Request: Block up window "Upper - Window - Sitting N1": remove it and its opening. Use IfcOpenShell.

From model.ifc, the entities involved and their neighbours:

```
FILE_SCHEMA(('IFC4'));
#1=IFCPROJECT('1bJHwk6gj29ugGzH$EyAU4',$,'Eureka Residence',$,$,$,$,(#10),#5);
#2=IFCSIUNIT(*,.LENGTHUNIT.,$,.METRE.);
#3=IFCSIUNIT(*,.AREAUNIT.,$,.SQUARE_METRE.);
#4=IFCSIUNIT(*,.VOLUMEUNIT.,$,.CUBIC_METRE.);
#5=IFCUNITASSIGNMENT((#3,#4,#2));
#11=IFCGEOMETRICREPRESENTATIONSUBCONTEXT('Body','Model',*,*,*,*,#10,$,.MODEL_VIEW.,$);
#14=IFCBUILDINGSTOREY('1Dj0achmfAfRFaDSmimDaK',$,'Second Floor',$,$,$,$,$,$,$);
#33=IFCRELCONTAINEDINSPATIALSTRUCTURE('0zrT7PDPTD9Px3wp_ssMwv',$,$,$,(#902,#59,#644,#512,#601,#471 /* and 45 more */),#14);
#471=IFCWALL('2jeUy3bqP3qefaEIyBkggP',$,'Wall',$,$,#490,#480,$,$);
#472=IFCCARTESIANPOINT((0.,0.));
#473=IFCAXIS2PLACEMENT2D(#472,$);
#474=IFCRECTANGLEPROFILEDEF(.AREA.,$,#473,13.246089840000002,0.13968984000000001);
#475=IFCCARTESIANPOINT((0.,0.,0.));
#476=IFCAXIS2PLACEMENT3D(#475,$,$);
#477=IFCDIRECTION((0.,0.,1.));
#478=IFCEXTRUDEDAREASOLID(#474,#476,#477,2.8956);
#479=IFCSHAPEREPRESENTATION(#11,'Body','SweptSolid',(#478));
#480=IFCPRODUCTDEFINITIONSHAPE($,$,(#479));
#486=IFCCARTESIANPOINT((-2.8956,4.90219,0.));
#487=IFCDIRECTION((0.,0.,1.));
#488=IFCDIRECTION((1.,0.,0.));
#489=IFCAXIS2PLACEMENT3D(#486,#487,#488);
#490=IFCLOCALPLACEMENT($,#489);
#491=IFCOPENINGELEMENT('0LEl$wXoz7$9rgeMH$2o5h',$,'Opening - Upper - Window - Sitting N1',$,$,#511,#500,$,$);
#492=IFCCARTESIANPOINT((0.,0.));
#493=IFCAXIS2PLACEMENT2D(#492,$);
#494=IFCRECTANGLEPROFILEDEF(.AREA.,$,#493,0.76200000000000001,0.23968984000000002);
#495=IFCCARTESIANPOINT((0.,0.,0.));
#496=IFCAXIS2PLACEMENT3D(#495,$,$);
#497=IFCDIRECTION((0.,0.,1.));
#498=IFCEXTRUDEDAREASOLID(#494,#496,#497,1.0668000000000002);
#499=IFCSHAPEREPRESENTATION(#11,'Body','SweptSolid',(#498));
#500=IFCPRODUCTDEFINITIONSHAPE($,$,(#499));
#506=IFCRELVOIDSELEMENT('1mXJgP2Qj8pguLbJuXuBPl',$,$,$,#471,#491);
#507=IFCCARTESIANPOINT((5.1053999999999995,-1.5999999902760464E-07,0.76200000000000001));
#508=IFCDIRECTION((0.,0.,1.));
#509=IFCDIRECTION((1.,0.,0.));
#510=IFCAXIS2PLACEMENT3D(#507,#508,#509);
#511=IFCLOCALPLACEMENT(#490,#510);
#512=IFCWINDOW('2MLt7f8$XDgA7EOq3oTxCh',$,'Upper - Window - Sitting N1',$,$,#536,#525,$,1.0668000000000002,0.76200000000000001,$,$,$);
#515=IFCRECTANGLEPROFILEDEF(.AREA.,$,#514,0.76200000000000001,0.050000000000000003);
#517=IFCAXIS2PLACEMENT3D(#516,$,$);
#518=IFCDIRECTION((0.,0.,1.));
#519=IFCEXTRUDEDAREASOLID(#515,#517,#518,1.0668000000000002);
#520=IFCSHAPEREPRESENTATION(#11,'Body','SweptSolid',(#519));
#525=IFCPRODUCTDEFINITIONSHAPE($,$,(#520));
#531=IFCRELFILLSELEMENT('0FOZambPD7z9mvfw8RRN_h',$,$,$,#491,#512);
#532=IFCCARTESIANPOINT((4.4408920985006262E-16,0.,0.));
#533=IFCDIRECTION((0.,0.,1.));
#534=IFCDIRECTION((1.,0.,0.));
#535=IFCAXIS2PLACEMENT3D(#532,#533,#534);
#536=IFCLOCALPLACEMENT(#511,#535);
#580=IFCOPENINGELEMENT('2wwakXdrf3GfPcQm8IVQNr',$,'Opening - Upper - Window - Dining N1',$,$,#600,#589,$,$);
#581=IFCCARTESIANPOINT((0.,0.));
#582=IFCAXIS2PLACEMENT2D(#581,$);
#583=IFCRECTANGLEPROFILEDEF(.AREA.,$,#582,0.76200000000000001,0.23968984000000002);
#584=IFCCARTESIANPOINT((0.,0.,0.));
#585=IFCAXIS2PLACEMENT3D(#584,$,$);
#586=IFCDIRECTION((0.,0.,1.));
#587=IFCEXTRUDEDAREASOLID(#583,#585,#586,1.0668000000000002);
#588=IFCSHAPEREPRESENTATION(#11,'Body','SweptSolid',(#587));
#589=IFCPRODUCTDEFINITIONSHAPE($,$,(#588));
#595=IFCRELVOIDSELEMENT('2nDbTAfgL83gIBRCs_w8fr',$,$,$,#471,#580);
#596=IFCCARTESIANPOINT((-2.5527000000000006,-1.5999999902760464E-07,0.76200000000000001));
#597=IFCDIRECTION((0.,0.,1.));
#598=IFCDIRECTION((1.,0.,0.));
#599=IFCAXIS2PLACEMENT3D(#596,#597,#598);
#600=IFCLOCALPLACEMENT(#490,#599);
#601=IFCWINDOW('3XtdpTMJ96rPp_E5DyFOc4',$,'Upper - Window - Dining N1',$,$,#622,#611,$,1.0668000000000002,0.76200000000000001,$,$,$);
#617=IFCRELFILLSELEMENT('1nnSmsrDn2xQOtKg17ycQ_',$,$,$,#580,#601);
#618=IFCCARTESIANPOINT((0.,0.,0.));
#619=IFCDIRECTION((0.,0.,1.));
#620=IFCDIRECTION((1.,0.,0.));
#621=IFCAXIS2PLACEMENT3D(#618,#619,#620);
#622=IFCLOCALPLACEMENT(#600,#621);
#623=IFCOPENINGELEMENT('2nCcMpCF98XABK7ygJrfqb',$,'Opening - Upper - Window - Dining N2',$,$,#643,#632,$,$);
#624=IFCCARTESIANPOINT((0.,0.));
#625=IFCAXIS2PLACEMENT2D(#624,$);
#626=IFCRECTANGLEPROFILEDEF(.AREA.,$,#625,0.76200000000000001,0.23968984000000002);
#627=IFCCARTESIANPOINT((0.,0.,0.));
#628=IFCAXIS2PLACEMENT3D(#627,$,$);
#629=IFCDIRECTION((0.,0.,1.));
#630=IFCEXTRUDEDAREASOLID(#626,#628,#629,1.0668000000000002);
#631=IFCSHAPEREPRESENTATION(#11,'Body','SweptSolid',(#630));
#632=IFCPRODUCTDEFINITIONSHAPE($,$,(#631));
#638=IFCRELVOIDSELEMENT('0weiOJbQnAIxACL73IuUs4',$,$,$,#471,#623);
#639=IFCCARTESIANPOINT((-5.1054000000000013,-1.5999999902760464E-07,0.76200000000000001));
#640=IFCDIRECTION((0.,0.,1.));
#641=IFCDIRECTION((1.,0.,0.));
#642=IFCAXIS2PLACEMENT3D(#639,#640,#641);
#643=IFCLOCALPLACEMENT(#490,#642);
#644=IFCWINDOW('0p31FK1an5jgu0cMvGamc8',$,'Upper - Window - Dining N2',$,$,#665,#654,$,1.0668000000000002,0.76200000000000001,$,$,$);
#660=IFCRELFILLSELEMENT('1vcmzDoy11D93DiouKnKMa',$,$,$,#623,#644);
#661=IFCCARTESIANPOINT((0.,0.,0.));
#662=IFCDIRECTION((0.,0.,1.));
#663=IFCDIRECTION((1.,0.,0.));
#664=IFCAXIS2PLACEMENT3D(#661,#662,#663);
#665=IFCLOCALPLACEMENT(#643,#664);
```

```python
import ifcopenshell
import ifcopenshell.api.feature
import ifcopenshell.api.root
import ifcopenshell.geom
import ifcopenshell.util.shape

model = ifcopenshell.open("model.ifc")
settings = ifcopenshell.geom.settings()


def volume(element):
    """Net volume in cubic metres, openings subtracted."""
    shape = ifcopenshell.geom.create_shape(settings, element)
    return ifcopenshell.util.shape.get_volume(shape.geometry)


window = model.by_guid("2MLt7f8$XDgA7EOq3oTxCh")
opening = window.FillsVoids[0].RelatingOpeningElement
wall = opening.VoidsElements[0].RelatingBuildingElement
before = volume(wall)

ifcopenshell.api.root.remove_product(model, product=window)
ifcopenshell.api.feature.remove_feature(model, feature=opening)

after = volume(wall)

print(f"wall volume {before:.3f} -> {after:.3f} m3")

model.write("model_updated.ifc")
```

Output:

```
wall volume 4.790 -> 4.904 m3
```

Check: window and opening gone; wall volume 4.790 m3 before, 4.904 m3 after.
